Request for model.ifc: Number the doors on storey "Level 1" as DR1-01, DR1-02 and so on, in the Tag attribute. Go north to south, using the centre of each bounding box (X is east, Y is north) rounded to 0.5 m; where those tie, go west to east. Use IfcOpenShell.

First a look at what the model holds.

```python
import ifcopenshell
import ifcopenshell.util.element
import ifcopenshell.util.placement

model = ifcopenshell.open("model.ifc")
print(model.schema)
storey = next(s for s in model.by_type("IfcBuildingStorey") if s.Name == "Level 1")
doors = [e for e in ifcopenshell.util.element.get_decomposition(storey) if e.is_a("IfcDoor")]
for e in sorted(doors, key=lambda e: e.id()):
    origin = ifcopenshell.util.placement.get_local_placement(e.ObjectPlacement)[:3, 3]
    print(e.id(), e.Tag, e.Name, origin.round(2) + 0.0, sep=" | ")
```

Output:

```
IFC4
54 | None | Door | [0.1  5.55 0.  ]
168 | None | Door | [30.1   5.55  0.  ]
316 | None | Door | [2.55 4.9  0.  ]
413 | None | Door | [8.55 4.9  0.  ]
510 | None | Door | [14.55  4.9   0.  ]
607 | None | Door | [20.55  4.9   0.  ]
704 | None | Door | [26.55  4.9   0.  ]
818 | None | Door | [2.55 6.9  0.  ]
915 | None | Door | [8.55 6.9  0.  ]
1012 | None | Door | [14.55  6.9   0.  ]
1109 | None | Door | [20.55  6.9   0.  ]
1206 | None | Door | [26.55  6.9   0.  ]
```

```python
import ifcopenshell
import ifcopenshell.geom
import ifcopenshell.util.element
import ifcopenshell.util.shape

model = ifcopenshell.open("model.ifc")
settings = ifcopenshell.geom.settings()
settings.set("use-world-coords", True)


def centre(element):
    shape = ifcopenshell.geom.create_shape(settings, element)
    return ifcopenshell.util.shape.get_bbox_centroid(shape.geometry)


storey = next(s for s in model.by_type("IfcBuildingStorey") if s.Name == "Level 1")
doors = [e for e in ifcopenshell.util.element.get_decomposition(storey) if e.is_a("IfcDoor")]

# Insertion points can sit at a corner or the storey origin, so sort by the geometry (in metres).
centres = {e: centre(e) for e in doors}
doors.sort(key=lambda e: (-round(centres[e][1] / 0.5), centres[e][0]))

for i, e in enumerate(doors, start=1):
    number = f"DR1-{i:02d}"
    e.Tag = number
    print(e.id(), number)

model.write("model_edited.ifc")
```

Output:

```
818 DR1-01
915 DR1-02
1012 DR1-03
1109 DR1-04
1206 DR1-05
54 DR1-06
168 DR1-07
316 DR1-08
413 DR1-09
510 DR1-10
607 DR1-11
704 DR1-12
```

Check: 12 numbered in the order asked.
